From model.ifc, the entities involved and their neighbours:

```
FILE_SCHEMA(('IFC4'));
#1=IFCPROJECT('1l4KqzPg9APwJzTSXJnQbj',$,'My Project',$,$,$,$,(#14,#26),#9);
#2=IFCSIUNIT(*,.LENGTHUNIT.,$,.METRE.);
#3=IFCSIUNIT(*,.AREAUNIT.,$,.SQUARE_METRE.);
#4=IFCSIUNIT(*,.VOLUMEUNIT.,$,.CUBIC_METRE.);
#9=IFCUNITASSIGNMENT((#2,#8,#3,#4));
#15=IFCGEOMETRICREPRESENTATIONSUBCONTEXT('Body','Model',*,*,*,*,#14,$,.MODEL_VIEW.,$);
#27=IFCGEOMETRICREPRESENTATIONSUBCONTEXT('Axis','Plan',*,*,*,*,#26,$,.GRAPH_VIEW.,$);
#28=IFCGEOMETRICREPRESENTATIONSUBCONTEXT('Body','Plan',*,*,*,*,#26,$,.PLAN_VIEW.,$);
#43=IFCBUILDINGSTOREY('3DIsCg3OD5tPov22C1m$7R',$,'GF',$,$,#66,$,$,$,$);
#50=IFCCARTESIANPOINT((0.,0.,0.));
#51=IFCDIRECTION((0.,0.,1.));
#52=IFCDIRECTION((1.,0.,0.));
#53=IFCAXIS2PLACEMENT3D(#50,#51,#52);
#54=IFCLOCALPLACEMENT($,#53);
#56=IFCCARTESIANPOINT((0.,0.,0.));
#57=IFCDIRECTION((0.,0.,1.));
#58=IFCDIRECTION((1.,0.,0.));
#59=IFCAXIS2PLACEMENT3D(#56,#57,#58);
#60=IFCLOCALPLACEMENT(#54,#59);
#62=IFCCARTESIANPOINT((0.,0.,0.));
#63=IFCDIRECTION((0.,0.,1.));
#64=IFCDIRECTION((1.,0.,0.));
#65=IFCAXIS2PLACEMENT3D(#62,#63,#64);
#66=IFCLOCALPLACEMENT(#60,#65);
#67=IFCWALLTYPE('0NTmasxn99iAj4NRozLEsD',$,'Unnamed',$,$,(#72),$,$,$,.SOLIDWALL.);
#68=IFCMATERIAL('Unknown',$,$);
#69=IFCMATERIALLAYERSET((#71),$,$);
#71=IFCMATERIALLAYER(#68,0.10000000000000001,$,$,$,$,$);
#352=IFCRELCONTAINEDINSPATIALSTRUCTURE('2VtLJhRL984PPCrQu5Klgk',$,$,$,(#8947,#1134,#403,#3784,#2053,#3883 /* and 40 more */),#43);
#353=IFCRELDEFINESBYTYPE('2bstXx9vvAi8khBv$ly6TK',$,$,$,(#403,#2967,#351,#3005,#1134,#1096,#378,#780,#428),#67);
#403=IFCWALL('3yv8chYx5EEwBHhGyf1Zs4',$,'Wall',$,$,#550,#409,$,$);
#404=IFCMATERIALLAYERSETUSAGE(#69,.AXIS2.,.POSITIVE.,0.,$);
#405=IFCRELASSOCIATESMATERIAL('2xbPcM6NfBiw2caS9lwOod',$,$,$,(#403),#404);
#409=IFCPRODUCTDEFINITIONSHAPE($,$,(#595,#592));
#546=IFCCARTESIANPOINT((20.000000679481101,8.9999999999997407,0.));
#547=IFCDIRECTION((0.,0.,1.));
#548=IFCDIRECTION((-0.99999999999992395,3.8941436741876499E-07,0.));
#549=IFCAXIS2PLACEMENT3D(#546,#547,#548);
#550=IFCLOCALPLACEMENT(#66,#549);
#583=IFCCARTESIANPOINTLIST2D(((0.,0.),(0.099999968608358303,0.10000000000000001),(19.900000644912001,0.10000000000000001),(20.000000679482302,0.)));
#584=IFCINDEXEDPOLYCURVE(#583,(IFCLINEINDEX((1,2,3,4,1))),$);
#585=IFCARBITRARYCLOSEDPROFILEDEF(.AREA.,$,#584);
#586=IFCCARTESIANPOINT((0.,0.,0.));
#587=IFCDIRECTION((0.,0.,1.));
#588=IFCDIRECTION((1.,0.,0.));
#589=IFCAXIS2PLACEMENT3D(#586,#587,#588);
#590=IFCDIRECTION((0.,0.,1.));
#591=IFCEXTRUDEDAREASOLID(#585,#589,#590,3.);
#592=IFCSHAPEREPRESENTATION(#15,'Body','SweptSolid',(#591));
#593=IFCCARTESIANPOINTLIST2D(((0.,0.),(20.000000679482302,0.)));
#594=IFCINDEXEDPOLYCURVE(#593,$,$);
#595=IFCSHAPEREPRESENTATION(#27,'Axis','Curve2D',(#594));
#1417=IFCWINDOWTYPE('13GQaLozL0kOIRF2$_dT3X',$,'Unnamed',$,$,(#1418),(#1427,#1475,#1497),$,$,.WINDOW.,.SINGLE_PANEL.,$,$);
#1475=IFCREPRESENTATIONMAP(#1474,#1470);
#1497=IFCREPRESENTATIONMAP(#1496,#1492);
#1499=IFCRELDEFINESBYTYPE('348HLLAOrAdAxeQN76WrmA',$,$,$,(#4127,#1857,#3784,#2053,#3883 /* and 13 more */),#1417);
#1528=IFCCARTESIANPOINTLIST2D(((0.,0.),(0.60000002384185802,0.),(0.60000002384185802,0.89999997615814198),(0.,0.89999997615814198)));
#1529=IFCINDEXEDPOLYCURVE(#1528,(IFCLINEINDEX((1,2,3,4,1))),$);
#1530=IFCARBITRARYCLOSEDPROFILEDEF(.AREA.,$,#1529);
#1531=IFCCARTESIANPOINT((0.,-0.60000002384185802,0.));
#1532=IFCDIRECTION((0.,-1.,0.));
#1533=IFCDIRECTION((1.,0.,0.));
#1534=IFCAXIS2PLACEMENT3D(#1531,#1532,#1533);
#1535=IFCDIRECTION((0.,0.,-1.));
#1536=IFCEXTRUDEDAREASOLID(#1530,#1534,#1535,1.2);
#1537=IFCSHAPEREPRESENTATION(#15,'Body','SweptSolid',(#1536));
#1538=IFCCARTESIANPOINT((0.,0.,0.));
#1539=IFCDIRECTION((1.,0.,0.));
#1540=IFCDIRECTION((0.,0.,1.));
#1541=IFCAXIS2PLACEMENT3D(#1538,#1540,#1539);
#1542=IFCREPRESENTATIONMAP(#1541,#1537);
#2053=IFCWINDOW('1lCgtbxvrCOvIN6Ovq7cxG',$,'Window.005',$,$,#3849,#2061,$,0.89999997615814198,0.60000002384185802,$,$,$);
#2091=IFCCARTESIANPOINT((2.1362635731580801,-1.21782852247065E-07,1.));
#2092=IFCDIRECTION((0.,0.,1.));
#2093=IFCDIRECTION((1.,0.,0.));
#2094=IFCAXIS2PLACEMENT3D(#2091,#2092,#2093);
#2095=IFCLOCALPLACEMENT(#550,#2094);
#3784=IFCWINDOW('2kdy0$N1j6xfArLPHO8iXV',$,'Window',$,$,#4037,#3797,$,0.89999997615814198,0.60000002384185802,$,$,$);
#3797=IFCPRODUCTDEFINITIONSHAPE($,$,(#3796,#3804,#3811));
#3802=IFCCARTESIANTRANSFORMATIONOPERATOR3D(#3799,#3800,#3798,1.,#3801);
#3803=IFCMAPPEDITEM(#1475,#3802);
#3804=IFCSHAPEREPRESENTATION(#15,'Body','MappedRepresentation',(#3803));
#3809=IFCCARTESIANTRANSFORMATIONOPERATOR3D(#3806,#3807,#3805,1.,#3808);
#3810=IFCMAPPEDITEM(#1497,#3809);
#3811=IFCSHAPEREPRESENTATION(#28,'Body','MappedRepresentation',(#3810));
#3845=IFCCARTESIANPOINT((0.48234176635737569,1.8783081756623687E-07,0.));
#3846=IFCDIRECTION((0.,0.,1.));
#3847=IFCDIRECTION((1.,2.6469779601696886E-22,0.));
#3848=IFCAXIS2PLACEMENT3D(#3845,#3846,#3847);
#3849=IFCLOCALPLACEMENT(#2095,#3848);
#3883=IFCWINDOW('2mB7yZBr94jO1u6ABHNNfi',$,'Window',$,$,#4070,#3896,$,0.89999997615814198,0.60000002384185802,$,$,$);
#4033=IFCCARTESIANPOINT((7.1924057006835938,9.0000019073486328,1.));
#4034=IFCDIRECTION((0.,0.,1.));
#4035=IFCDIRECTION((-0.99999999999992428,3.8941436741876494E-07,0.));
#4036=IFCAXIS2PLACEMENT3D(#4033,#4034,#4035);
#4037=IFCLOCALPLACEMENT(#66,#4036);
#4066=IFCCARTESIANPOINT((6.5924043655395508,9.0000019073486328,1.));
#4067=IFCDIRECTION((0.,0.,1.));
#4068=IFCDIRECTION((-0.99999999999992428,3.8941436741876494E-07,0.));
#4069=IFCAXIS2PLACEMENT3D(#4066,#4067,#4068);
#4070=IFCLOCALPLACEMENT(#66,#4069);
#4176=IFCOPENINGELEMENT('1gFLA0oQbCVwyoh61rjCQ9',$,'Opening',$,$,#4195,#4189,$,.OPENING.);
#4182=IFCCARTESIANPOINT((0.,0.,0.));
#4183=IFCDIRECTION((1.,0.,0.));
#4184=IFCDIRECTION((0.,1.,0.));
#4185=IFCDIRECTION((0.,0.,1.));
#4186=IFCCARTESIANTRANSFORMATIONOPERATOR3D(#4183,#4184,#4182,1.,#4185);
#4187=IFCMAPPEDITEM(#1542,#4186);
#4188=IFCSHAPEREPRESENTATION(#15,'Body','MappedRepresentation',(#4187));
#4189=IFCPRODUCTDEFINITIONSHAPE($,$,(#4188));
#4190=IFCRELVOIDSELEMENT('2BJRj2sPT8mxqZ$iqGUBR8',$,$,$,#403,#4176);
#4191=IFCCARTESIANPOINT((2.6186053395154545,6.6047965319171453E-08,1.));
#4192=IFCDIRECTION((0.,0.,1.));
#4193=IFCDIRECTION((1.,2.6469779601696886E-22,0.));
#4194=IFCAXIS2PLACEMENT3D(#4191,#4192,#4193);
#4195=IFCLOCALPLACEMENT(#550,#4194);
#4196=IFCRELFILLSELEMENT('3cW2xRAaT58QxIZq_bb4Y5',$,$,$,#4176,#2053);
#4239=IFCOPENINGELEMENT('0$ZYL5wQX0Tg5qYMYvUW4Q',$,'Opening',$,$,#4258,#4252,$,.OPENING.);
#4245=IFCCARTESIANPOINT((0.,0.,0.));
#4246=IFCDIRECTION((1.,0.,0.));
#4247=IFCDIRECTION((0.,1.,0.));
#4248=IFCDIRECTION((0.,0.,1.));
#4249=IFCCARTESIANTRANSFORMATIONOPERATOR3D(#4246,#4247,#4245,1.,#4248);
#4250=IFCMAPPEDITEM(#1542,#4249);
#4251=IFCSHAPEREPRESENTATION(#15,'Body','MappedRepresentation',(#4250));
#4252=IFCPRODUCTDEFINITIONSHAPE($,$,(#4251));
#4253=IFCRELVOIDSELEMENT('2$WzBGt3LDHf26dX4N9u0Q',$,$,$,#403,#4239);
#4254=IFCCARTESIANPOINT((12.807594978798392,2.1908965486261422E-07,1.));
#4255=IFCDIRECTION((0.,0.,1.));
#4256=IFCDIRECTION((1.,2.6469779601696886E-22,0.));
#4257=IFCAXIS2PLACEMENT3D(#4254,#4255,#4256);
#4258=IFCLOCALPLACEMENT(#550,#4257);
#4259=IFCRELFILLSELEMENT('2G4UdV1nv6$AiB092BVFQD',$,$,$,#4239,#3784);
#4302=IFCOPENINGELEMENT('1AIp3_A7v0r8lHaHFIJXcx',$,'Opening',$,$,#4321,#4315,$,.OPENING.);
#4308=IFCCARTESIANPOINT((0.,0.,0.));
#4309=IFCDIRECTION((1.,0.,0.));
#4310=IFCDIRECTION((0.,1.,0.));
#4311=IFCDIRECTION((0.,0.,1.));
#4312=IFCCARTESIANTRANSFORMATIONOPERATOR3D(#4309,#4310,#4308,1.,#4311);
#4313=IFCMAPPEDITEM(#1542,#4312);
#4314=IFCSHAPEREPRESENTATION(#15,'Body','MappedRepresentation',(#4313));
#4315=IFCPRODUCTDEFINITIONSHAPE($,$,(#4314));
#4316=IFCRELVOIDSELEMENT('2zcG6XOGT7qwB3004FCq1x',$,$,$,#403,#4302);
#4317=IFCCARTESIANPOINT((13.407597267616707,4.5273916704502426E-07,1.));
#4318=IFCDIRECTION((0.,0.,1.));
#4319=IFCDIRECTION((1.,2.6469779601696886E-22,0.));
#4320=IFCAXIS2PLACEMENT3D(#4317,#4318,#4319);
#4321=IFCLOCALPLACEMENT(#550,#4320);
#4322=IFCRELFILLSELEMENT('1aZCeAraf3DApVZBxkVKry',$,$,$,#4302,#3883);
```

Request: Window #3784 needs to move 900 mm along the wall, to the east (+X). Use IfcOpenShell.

```python
import ifcopenshell
import ifcopenshell.api.geometry
import ifcopenshell.util.placement
import ifcopenshell.util.unit

model = ifcopenshell.open("model.ifc")
unit_scale = ifcopenshell.util.unit.calculate_unit_scale(model)

window = model.by_guid("2kdy0$N1j6xfArLPHO8iXV")
opening = window.FillsVoids[0].RelatingOpeningElement
wall = opening.VoidsElements[0].RelatingBuildingElement

wall_matrix = ifcopenshell.util.placement.get_local_placement(wall.ObjectPlacement)
shift = wall_matrix[:3, 0] * -0.9 / unit_scale
before = ifcopenshell.util.placement.get_local_placement(window.ObjectPlacement)[:3, 3].copy()

# The window is not placed relative to its opening, so move both.
for product in (opening, window):
    matrix = ifcopenshell.util.placement.get_local_placement(product.ObjectPlacement)
    matrix[:3, 3] += shift
    ifcopenshell.api.geometry.edit_object_placement(model, product=product, matrix=matrix, is_si=False)

after = ifcopenshell.util.placement.get_local_placement(window.ObjectPlacement)[:3, 3]
print("window moved by", (after - before).round(3) + 0.0)

model.write("model_edited.ifc")
```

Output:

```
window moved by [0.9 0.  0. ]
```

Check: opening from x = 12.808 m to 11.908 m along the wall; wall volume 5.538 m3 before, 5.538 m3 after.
